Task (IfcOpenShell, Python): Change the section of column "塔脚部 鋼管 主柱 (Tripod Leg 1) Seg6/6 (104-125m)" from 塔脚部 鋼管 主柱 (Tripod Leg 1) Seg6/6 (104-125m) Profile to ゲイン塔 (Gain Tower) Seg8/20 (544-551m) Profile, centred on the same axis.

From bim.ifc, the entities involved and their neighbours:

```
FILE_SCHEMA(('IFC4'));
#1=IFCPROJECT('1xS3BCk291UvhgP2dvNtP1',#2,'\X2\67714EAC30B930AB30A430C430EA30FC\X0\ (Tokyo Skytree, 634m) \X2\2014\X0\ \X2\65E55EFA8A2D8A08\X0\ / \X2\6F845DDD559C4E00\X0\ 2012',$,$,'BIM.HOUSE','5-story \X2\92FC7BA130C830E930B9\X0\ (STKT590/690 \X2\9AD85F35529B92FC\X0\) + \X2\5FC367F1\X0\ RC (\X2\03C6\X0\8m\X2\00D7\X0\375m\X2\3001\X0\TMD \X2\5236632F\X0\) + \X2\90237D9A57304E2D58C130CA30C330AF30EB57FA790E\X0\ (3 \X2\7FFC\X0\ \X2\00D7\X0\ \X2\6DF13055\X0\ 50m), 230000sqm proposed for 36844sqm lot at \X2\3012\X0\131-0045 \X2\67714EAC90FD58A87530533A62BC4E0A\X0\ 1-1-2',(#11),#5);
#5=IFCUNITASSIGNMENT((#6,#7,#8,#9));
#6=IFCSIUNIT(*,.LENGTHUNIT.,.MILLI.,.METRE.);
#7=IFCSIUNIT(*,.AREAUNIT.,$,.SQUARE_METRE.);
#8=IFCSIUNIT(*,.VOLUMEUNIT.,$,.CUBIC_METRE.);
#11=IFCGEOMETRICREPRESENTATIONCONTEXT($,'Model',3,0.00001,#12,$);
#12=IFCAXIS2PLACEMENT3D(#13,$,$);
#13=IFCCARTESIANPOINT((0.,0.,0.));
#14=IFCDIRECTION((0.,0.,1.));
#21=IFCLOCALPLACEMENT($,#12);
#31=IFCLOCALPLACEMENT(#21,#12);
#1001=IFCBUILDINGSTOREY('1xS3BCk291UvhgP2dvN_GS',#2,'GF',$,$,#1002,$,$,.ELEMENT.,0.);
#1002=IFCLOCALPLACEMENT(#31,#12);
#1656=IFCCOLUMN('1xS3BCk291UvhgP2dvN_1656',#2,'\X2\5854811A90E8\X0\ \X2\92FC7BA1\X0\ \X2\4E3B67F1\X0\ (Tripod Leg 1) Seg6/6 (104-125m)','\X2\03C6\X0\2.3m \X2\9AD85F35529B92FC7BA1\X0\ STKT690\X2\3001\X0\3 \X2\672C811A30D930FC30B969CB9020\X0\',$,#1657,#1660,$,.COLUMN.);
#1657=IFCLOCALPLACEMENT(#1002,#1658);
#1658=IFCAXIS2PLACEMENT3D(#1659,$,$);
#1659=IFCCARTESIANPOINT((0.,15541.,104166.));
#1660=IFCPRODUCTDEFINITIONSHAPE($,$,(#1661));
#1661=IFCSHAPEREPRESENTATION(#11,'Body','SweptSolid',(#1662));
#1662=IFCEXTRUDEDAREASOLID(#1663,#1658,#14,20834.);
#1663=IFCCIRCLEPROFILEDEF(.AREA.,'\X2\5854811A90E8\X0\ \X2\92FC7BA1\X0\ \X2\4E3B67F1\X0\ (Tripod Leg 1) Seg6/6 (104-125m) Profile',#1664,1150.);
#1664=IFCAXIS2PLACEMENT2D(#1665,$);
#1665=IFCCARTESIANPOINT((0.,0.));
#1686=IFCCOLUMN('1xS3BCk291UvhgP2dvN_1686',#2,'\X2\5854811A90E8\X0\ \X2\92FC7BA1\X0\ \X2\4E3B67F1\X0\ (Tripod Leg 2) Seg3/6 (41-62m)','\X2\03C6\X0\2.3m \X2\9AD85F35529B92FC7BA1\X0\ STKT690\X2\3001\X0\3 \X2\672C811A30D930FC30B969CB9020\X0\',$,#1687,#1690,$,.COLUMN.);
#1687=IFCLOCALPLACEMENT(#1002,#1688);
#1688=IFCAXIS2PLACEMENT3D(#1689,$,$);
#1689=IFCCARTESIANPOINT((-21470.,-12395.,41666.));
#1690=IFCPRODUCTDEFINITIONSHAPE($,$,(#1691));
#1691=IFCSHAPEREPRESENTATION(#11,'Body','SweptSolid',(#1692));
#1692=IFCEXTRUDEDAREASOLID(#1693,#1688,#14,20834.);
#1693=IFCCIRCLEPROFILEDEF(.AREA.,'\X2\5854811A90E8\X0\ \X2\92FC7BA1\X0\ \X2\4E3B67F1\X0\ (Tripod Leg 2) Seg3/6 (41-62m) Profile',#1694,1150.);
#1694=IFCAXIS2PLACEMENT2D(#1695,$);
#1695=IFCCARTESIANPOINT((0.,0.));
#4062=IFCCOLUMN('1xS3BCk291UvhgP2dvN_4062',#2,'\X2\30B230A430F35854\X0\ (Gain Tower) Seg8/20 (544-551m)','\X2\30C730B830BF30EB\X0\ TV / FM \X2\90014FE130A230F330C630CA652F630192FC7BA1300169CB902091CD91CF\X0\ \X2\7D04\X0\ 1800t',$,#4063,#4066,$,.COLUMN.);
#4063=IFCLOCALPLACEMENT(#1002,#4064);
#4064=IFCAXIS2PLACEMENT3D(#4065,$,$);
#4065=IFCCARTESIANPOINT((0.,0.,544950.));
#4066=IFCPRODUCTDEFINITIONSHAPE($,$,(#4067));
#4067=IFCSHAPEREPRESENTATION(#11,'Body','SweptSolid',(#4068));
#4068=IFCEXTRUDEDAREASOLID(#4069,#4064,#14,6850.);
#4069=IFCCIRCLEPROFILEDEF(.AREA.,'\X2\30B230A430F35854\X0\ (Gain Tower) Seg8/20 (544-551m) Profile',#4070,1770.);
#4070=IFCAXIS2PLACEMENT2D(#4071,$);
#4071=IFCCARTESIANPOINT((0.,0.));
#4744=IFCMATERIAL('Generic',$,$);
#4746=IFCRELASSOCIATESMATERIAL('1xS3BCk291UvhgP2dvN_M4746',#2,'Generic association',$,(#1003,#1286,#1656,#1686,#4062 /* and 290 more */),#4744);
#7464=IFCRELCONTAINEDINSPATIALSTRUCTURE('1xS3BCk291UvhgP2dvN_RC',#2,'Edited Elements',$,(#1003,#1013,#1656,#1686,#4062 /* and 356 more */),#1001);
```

```python
import ifcopenshell
import ifcopenshell.util.element

model = ifcopenshell.open("bim.ifc")

member = model.by_guid("1xS3BCk291UvhgP2dvN_1656")
source = next(p for p in model.by_type("IfcCircleProfileDef") if p.ProfileName == "ゲイン塔 (Gain Tower) Seg8/20 (544-551m) Profile")

body = next(r for r in member.Representation.Representations if r.RepresentationIdentifier == "Body")
solid = body.Items[0]
old_profile = solid.SweptArea

# Copy the section's sizes but keep this member's own profile position.
profile = ifcopenshell.util.element.copy(model, source)
profile.Position = old_profile.Position
solid.SweptArea = profile
if not model.get_total_inverses(old_profile):
    ifcopenshell.util.element.remove_deep2(model, old_profile)

print(solid.SweptArea)

model.write("bim_edited.ifc")
```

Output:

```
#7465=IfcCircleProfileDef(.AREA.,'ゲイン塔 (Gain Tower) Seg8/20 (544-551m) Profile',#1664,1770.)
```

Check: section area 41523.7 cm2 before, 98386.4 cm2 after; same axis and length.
